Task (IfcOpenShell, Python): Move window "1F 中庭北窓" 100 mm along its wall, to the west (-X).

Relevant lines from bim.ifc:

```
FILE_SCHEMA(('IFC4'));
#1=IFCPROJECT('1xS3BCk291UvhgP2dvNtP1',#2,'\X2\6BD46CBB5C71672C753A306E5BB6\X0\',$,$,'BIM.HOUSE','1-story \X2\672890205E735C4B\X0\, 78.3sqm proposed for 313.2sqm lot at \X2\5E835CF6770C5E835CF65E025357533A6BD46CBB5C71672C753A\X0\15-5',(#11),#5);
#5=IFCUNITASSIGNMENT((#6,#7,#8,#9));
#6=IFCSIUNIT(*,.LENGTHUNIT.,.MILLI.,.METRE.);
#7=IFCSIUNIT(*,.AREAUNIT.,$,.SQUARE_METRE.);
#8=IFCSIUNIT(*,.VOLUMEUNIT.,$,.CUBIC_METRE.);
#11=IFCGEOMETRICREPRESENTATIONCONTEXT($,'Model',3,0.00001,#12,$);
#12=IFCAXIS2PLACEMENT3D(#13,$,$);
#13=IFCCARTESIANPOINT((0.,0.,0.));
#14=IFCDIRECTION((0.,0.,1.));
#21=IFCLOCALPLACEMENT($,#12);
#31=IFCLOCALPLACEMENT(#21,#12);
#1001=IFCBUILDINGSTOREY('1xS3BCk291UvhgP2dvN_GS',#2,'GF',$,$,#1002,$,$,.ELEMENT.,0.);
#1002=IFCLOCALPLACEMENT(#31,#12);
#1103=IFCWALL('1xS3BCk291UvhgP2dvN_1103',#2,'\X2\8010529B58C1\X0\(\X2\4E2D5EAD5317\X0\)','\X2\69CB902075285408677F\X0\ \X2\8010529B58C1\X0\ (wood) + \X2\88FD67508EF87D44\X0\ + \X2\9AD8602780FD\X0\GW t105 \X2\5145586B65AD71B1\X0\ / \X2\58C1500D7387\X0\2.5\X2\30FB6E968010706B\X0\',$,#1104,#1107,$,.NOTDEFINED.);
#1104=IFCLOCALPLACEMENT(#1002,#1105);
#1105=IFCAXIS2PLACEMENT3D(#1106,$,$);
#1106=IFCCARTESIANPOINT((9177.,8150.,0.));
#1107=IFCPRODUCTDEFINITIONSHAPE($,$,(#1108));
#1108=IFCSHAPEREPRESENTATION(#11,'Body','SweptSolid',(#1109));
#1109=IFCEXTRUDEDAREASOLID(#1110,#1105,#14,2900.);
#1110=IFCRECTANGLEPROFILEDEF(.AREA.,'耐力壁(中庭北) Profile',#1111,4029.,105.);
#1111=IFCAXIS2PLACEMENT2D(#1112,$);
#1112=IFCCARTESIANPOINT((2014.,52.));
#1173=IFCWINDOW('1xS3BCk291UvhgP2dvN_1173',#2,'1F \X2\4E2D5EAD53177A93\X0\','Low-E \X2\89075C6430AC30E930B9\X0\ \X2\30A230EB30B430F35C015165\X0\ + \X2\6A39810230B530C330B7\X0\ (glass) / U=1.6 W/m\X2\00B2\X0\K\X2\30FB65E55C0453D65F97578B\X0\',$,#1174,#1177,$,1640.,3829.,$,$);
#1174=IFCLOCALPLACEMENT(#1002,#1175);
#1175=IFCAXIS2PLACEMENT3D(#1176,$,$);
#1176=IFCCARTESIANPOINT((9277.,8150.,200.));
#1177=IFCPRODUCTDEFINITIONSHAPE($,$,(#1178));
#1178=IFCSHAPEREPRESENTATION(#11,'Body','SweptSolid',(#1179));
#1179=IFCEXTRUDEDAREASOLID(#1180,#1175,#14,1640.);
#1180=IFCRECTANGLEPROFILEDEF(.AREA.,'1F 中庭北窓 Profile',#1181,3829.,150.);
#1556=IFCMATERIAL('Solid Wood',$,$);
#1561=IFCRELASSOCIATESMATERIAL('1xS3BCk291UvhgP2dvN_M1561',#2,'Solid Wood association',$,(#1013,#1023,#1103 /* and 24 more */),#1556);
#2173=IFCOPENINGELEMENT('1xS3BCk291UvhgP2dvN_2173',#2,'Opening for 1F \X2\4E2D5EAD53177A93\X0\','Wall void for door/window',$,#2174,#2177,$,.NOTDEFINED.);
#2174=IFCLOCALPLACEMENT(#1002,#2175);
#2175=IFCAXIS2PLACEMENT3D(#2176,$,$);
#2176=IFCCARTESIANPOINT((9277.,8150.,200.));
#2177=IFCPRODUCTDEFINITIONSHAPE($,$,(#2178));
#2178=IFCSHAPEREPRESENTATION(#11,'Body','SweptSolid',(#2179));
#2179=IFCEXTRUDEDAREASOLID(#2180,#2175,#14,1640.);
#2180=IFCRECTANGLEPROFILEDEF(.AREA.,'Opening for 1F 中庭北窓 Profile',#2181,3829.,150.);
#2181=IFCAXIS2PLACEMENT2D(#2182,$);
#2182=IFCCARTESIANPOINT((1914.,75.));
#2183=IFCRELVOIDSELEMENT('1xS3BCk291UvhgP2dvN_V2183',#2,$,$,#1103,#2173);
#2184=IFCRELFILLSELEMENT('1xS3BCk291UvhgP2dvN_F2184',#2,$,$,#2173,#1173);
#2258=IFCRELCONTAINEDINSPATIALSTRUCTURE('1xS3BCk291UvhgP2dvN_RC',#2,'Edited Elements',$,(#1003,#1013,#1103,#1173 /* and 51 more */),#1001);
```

```python
import ifcopenshell
import ifcopenshell.api.geometry
import ifcopenshell.util.placement

model = ifcopenshell.open("bim.ifc")

window = model.by_id(1173)
opening = window.FillsVoids[0].RelatingOpeningElement
wall = opening.VoidsElements[0].RelatingBuildingElement

wall_matrix = ifcopenshell.util.placement.get_local_placement(wall.ObjectPlacement)
shift = wall_matrix[:3, 0] * -100.0
before = ifcopenshell.util.placement.get_local_placement(window.ObjectPlacement)[:3, 3].copy()

# The window is not placed relative to its opening, so move both.
for product in (opening, window):
    matrix = ifcopenshell.util.placement.get_local_placement(product.ObjectPlacement)
    matrix[:3, 3] += shift
    ifcopenshell.api.geometry.edit_object_placement(model, product=product, matrix=matrix, is_si=False)

after = ifcopenshell.util.placement.get_local_placement(window.ObjectPlacement)[:3, 3]
print("window moved by", (after - before).round(3) + 0.0)

model.write("bim_updated.ifc")
```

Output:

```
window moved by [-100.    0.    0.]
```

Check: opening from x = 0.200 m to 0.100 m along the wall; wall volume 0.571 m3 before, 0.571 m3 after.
